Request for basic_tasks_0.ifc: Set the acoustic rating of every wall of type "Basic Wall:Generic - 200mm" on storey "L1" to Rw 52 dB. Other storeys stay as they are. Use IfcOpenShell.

First a look at what the model holds.

```python
import ifcopenshell
import ifcopenshell.util.element

model = ifcopenshell.open("basic_tasks_0.ifc")
print(model.schema)
storey = next(s for s in model.by_type("IfcBuildingStorey") if s.Name == "L1")
walls = [e for e in ifcopenshell.util.element.get_decomposition(storey) if e.is_a("IfcWall")]
seen = {}
for e in walls:
    element_type = ifcopenshell.util.element.get_type(e)
    key = (element_type.Name if element_type != e and element_type else None, ifcopenshell.util.element.get_pset(e, "Pset_WallCommon", "AcousticRating"))
    seen[key] = seen.get(key, 0) + 1
for (name, value), count in sorted(seen.items(), key=str):
    print(count, "x", name, "|", value)
```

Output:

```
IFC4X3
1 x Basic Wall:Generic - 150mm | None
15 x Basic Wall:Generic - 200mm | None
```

```python
import ifcopenshell
import ifcopenshell.api.pset
import ifcopenshell.util.element

model = ifcopenshell.open("basic_tasks_0.ifc")

storey = next(s for s in model.by_type("IfcBuildingStorey") if s.Name == "L1")
walls = [e for e in ifcopenshell.util.element.get_decomposition(storey) if e.is_a("IfcWall")]

count = 0
for e in walls:
    element_type = ifcopenshell.util.element.get_type(e)
    if element_type in (None, e) or element_type.Name != "Basic Wall:Generic - 200mm":
        continue
    # add_pset returns the element's existing set when there is one.
    pset = ifcopenshell.api.pset.add_pset(model, product=e, name="Pset_WallCommon")
    ifcopenshell.api.pset.edit_pset(model, pset=pset, properties={"AcousticRating": "Rw 52 dB"})
    count += 1

print(count, "walls updated")

model.write("basic_tasks_0-out.ifc")
```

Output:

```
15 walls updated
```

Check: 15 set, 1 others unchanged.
